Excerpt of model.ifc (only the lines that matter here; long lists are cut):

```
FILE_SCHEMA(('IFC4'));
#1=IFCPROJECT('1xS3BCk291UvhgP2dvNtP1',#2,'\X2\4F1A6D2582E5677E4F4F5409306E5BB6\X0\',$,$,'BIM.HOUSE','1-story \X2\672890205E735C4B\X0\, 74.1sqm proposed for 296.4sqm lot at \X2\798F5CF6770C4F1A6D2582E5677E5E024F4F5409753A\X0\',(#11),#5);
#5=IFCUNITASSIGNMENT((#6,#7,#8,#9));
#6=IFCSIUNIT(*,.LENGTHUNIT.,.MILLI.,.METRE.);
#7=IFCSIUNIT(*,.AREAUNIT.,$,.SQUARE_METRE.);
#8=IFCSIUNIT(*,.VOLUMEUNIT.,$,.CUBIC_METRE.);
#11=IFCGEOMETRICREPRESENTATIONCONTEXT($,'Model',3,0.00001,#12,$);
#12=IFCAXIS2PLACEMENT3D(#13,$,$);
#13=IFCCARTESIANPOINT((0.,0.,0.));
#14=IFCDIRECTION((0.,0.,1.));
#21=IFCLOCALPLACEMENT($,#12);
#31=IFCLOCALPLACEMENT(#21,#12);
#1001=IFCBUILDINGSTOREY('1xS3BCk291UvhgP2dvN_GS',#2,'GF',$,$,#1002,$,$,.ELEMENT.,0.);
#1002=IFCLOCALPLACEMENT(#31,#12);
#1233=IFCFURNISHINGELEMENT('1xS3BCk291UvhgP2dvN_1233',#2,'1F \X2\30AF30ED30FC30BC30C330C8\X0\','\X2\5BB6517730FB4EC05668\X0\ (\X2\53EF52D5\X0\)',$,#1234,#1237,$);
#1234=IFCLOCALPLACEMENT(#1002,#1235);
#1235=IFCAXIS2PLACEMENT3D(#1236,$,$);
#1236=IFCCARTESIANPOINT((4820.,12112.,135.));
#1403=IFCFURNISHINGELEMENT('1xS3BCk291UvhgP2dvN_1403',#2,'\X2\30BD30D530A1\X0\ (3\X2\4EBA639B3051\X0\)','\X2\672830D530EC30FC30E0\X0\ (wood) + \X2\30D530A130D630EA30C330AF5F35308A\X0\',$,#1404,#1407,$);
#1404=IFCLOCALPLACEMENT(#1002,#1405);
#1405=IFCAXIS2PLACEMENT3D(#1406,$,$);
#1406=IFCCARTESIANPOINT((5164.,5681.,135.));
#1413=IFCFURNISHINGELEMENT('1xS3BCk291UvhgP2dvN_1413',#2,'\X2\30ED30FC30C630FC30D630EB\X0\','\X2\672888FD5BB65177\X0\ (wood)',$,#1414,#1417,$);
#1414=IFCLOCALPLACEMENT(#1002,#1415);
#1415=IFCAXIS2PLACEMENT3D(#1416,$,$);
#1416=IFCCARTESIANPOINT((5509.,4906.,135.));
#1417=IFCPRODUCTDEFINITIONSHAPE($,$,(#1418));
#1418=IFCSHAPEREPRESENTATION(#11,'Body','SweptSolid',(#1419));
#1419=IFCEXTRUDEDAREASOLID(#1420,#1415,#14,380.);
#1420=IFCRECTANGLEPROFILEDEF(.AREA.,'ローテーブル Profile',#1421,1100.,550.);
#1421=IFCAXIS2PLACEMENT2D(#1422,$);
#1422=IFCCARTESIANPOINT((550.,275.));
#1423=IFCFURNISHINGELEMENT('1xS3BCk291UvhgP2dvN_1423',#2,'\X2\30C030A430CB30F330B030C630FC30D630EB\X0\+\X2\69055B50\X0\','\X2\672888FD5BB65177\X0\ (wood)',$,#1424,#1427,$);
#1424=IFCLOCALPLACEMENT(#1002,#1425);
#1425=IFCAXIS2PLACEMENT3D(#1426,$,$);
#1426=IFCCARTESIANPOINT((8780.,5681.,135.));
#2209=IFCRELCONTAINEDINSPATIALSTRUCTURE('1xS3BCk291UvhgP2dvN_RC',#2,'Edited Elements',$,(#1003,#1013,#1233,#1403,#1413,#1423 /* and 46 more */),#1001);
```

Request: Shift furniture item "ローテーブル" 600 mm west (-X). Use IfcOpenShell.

```python
import ifcopenshell
import ifcopenshell.api.geometry
import ifcopenshell.util.placement
import ifcopenshell.util.unit

model = ifcopenshell.open("model.ifc")
unit_scale = ifcopenshell.util.unit.calculate_unit_scale(model)

item = model.by_id(1413)
matrix = ifcopenshell.util.placement.get_local_placement(item.ObjectPlacement)
matrix[0, 3] -= 0.6 / unit_scale
ifcopenshell.api.geometry.edit_object_placement(model, product=item, matrix=matrix, is_si=False)

print(ifcopenshell.util.placement.get_local_placement(item.ObjectPlacement).round(3) + 0.0)

model.write("model-out.ifc")
```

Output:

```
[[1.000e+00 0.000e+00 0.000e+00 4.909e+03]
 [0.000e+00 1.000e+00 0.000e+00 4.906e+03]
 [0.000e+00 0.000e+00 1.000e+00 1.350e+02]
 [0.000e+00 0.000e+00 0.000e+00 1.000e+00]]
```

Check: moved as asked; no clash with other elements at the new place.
